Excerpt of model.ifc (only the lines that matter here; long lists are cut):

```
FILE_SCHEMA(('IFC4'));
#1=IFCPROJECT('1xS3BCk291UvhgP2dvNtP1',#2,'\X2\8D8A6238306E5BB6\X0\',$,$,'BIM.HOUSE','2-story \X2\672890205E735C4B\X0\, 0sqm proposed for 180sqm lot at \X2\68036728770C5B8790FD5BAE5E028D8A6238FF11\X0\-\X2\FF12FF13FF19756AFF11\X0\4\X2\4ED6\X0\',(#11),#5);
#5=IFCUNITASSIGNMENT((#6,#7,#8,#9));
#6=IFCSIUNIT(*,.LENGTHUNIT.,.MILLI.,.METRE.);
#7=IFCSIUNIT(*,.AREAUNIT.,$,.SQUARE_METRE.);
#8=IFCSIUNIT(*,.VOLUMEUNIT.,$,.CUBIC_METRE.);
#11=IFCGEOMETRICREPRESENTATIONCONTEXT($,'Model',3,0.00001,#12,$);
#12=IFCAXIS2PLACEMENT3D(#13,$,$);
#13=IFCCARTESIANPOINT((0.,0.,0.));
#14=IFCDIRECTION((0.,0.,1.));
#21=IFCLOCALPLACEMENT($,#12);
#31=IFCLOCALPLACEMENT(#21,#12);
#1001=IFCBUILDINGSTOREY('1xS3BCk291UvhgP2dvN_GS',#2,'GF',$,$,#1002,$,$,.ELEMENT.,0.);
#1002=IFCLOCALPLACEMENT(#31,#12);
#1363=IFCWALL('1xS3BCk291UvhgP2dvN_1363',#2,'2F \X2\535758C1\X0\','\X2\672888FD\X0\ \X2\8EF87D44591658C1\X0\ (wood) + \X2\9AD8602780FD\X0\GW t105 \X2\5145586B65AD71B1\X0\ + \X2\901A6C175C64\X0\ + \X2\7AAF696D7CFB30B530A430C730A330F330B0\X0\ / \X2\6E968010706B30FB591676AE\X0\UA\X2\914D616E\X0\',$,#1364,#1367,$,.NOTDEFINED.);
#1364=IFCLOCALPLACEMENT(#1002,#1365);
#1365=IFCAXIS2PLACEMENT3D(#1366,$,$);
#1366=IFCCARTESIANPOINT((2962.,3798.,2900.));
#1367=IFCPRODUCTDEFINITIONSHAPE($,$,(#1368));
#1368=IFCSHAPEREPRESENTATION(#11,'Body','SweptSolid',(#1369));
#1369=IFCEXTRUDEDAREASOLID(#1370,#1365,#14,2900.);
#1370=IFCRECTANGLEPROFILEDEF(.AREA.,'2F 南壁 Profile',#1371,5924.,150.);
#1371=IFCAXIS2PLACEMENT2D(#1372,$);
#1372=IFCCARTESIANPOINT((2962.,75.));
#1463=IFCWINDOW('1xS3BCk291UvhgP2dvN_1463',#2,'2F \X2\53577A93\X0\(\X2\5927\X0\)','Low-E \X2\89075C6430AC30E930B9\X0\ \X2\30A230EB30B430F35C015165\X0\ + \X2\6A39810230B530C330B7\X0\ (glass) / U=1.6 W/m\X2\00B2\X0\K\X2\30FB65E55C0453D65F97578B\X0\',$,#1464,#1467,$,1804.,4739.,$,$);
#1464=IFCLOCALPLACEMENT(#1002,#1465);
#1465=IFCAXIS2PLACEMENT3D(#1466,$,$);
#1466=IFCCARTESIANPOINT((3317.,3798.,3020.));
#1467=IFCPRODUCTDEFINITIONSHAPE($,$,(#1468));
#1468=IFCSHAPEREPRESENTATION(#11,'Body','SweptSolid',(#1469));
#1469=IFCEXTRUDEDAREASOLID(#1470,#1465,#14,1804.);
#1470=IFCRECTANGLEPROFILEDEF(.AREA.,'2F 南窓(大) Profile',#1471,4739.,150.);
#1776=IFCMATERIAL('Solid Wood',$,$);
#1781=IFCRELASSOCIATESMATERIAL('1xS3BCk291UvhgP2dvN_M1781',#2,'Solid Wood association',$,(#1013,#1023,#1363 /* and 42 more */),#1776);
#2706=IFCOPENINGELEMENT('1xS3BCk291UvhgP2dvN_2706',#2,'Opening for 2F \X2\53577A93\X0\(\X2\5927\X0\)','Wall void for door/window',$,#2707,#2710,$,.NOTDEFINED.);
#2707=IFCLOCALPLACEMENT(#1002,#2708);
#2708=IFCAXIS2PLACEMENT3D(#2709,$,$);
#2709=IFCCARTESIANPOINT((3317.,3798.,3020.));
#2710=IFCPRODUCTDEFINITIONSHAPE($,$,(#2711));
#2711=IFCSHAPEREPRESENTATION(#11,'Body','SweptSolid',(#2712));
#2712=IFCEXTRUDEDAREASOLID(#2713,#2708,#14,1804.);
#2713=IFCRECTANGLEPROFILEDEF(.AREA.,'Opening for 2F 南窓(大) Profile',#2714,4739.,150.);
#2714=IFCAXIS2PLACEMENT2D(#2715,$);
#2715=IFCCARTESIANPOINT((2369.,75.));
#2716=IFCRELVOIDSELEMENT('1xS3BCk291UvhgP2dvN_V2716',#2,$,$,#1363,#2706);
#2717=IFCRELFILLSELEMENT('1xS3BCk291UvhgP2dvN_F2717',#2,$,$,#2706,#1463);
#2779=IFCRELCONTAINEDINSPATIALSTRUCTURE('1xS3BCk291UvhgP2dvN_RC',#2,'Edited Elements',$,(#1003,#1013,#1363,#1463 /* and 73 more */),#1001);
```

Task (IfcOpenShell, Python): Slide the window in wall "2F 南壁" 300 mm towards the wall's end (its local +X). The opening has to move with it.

```python
import ifcopenshell
import ifcopenshell.api.geometry
import ifcopenshell.util.placement
import ifcopenshell.util.unit

model = ifcopenshell.open("model.ifc")
unit_scale = ifcopenshell.util.unit.calculate_unit_scale(model)

window = model.by_guid("1xS3BCk291UvhgP2dvN_1463")
opening = window.FillsVoids[0].RelatingOpeningElement
wall = opening.VoidsElements[0].RelatingBuildingElement

wall_matrix = ifcopenshell.util.placement.get_local_placement(wall.ObjectPlacement)
shift = wall_matrix[:3, 0] * 0.3 / unit_scale
before = ifcopenshell.util.placement.get_local_placement(window.ObjectPlacement)[:3, 3].copy()

# The window is not placed relative to its opening, so move both.
for product in (opening, window):
    matrix = ifcopenshell.util.placement.get_local_placement(product.ObjectPlacement)
    matrix[:3, 3] += shift
    ifcopenshell.api.geometry.edit_object_placement(model, product=product, matrix=matrix, is_si=False)

after = ifcopenshell.util.placement.get_local_placement(window.ObjectPlacement)[:3, 3]
print("window moved by", (after - before).round(3) + 0.0)

model.write("model_rev.ifc")
```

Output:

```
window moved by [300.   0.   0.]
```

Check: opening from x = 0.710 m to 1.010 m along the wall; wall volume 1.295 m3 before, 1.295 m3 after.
